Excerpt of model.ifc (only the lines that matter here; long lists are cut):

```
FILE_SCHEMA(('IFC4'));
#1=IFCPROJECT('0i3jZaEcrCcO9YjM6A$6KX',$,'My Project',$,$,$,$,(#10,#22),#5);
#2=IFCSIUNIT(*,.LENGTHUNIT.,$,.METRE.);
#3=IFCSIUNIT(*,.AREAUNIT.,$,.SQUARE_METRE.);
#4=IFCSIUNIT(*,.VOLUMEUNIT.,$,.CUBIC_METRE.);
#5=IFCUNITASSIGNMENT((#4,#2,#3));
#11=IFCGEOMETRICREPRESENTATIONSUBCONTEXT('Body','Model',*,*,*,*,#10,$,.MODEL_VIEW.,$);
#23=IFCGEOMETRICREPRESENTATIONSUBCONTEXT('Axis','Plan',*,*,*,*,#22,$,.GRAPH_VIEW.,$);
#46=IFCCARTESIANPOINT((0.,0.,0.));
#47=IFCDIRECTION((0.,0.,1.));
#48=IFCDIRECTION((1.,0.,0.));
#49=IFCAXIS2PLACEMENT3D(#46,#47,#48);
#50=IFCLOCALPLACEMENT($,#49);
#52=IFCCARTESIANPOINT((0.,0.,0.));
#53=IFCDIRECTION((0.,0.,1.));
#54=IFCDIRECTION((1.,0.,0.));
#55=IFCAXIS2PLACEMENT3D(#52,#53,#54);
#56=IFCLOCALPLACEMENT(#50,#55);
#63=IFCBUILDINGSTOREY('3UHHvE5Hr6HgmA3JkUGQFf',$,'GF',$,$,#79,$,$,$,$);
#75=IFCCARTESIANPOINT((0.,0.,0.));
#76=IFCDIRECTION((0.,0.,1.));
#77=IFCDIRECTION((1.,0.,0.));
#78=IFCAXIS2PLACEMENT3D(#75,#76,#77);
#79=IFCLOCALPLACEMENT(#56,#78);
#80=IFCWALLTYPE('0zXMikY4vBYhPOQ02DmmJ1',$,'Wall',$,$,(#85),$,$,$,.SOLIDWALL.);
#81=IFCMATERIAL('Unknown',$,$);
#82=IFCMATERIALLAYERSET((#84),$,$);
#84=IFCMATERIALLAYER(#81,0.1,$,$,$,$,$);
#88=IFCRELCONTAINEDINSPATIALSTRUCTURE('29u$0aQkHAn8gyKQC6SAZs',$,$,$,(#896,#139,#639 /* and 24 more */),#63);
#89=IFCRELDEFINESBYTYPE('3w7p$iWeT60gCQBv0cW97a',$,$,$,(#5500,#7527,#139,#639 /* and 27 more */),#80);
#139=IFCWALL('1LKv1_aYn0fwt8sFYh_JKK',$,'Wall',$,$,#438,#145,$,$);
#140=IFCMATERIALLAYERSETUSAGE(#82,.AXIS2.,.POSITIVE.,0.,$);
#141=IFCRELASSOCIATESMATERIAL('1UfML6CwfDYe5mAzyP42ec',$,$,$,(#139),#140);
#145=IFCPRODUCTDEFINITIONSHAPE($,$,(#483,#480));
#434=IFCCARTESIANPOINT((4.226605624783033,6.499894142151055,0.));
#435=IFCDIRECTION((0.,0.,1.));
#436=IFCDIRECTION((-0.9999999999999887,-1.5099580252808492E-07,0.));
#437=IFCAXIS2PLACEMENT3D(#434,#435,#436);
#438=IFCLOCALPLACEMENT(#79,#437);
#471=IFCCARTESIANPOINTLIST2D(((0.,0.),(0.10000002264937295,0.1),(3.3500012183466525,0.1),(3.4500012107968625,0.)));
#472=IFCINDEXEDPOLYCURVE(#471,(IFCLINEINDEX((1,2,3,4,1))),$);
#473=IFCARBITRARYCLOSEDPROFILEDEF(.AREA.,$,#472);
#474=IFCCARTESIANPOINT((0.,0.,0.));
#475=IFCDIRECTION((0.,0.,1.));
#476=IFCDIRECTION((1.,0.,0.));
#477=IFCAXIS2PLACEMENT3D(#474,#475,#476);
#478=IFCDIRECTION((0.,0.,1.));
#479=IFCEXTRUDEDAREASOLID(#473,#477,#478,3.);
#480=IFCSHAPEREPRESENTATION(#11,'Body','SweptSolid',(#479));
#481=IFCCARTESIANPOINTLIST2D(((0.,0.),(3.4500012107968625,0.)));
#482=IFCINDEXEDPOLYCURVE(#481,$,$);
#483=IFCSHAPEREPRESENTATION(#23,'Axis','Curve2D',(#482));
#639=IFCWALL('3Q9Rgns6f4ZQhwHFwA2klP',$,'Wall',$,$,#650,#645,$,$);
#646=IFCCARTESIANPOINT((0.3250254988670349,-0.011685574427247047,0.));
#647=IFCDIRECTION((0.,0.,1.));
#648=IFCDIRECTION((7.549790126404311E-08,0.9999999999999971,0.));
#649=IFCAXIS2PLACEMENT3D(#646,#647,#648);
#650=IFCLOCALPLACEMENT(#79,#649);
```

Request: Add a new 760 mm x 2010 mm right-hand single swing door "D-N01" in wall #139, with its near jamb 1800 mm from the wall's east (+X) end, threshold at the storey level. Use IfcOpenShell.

```python
import numpy as np
import ifcopenshell
import ifcopenshell.api.feature
import ifcopenshell.api.geometry
import ifcopenshell.api.root
import ifcopenshell.api.spatial
import ifcopenshell.geom
import ifcopenshell.util.element
import ifcopenshell.util.placement
import ifcopenshell.util.representation
import ifcopenshell.util.shape
import ifcopenshell.util.unit

model = ifcopenshell.open("model.ifc")
unit_scale = ifcopenshell.util.unit.calculate_unit_scale(model)
settings = ifcopenshell.geom.settings()


def volume(element):
    """Net volume in cubic metres, openings subtracted."""
    shape = ifcopenshell.geom.create_shape(settings, element)
    return ifcopenshell.util.shape.get_volume(shape.geometry)


wall = model.by_guid("1LKv1_aYn0fwt8sFYh_JKK")
storey = ifcopenshell.util.element.get_container(wall, ifc_class="IfcBuildingStorey")
context = ifcopenshell.util.representation.get_context(model, "Model", "Body", "MODEL_VIEW")
before = volume(wall)

width, height, from_end, sill = 0.76, 2.01, 1.8, 0.0  # metres

# The wall runs along its own X axis, and the end named is its -X end.
wall_shape = ifcopenshell.geom.create_shape(settings, wall)
x, y, z = ifcopenshell.util.shape.get_vertices(wall_shape.geometry).T
start = x.min() + from_end
face, thickness = float(y.min()), float(y.max() - y.min())
wall_matrix = ifcopenshell.util.placement.get_local_placement(wall.ObjectPlacement)
level = ifcopenshell.util.placement.get_local_placement(storey.ObjectPlacement)[2, 3]


def in_wall(x, y):
    """Placement at x, y metres in the wall's axes, at sill height."""
    matrix = wall_matrix.copy()
    matrix[:, 3] = wall_matrix @ np.array([x / unit_scale, y / unit_scale, 0.0, 1.0])
    matrix[2, 3] = level + sill / unit_scale
    return matrix


# Opening: a box that overshoots both wall faces by 50 mm.
opening = ifcopenshell.api.root.create_entity(model, ifc_class="IfcOpeningElement", predefined_type="OPENING")
box = ifcopenshell.api.geometry.add_wall_representation(
    model, context=context, length=width, height=height, thickness=thickness + 0.1
)
ifcopenshell.api.geometry.assign_representation(model, product=opening, representation=box)
ifcopenshell.api.geometry.edit_object_placement(model, product=opening, matrix=in_wall(start, face - 0.05), is_si=False)
ifcopenshell.api.feature.add_feature(model, feature=opening, element=wall)

door = ifcopenshell.api.root.create_entity(model, ifc_class="IfcDoor", name="D-N01", predefined_type="DOOR")
door.OverallWidth, door.OverallHeight = width / unit_scale, height / unit_scale
door.OperationType = "SINGLE_SWING_RIGHT"
body = ifcopenshell.api.geometry.add_door_representation(
    model,
    context=context,
    overall_width=door.OverallWidth,
    overall_height=door.OverallHeight,
    operation_type="SINGLE_SWING_RIGHT",
    lining_properties={"LiningDepth": thickness / unit_scale, "ThresholdDepth": thickness / unit_scale},
)
ifcopenshell.api.geometry.assign_representation(model, product=door, representation=body)
ifcopenshell.api.spatial.assign_container(model, products=[door], relating_structure=storey)
ifcopenshell.api.feature.add_filling(model, opening=opening, element=door)

# The lining spans the wall, so the door starts at the wall face.
ifcopenshell.api.geometry.edit_object_placement(model, product=door, matrix=in_wall(start, face), is_si=False)

after = volume(wall)

print(f"wall volume {before:.3f} -> {after:.3f} m3")

model.write("model_edited.ifc")
```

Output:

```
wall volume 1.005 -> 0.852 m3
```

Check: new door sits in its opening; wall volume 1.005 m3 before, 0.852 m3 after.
